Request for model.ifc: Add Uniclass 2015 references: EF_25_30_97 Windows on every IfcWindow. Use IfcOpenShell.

First a look at what the model holds.

```python
import ifcopenshell

model = ifcopenshell.open("model.ifc")
print(model.schema)
print("classifications:", [c.Name for c in model.by_type("IfcClassification")])
for ifc_class in ("IfcDoor", "IfcRoof", "IfcStair", "IfcWall", "IfcWindow"):
    print(ifc_class, len(model.by_type(ifc_class)))
```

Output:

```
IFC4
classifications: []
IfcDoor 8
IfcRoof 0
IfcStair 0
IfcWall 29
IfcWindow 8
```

```python
import ifcopenshell
import ifcopenshell.api.classification

model = ifcopenshell.open("model.ifc")

system = ifcopenshell.api.classification.add_classification(model, classification="Uniclass 2015")

codes = {
    "IfcWindow": ("EF_25_30_97", "Windows"),
}
for ifc_class, (code, name) in codes.items():
    products = model.by_type(ifc_class)
    ifcopenshell.api.classification.add_reference(
        model, products=products, classification=system, identification=code, name=name
    )
    print(code, len(products))

model.write("model_edited.ifc")
```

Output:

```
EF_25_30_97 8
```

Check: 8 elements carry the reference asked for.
